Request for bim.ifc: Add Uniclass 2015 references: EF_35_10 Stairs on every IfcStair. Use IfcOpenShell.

First a look at what the model holds.

```python
import ifcopenshell

model = ifcopenshell.open("bim.ifc")
print(model.schema)
print("classifications:", [c.Name for c in model.by_type("IfcClassification")])
for ifc_class in ("IfcDoor", "IfcRoof", "IfcStair", "IfcWall", "IfcWindow"):
    print(ifc_class, len(model.by_type(ifc_class)))
```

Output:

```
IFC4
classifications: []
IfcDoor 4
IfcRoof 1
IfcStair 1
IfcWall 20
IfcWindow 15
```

```python
import ifcopenshell
import ifcopenshell.api.classification

model = ifcopenshell.open("bim.ifc")

system = ifcopenshell.api.classification.add_classification(model, classification="Uniclass 2015")

codes = {
    "IfcStair": ("EF_35_10", "Stairs"),
}
for ifc_class, (code, name) in codes.items():
    products = model.by_type(ifc_class)
    ifcopenshell.api.classification.add_reference(
        model, products=products, classification=system, identification=code, name=name
    )
    print(code, len(products))

model.write("bim_rev.ifc")
```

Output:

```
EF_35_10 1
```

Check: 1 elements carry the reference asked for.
